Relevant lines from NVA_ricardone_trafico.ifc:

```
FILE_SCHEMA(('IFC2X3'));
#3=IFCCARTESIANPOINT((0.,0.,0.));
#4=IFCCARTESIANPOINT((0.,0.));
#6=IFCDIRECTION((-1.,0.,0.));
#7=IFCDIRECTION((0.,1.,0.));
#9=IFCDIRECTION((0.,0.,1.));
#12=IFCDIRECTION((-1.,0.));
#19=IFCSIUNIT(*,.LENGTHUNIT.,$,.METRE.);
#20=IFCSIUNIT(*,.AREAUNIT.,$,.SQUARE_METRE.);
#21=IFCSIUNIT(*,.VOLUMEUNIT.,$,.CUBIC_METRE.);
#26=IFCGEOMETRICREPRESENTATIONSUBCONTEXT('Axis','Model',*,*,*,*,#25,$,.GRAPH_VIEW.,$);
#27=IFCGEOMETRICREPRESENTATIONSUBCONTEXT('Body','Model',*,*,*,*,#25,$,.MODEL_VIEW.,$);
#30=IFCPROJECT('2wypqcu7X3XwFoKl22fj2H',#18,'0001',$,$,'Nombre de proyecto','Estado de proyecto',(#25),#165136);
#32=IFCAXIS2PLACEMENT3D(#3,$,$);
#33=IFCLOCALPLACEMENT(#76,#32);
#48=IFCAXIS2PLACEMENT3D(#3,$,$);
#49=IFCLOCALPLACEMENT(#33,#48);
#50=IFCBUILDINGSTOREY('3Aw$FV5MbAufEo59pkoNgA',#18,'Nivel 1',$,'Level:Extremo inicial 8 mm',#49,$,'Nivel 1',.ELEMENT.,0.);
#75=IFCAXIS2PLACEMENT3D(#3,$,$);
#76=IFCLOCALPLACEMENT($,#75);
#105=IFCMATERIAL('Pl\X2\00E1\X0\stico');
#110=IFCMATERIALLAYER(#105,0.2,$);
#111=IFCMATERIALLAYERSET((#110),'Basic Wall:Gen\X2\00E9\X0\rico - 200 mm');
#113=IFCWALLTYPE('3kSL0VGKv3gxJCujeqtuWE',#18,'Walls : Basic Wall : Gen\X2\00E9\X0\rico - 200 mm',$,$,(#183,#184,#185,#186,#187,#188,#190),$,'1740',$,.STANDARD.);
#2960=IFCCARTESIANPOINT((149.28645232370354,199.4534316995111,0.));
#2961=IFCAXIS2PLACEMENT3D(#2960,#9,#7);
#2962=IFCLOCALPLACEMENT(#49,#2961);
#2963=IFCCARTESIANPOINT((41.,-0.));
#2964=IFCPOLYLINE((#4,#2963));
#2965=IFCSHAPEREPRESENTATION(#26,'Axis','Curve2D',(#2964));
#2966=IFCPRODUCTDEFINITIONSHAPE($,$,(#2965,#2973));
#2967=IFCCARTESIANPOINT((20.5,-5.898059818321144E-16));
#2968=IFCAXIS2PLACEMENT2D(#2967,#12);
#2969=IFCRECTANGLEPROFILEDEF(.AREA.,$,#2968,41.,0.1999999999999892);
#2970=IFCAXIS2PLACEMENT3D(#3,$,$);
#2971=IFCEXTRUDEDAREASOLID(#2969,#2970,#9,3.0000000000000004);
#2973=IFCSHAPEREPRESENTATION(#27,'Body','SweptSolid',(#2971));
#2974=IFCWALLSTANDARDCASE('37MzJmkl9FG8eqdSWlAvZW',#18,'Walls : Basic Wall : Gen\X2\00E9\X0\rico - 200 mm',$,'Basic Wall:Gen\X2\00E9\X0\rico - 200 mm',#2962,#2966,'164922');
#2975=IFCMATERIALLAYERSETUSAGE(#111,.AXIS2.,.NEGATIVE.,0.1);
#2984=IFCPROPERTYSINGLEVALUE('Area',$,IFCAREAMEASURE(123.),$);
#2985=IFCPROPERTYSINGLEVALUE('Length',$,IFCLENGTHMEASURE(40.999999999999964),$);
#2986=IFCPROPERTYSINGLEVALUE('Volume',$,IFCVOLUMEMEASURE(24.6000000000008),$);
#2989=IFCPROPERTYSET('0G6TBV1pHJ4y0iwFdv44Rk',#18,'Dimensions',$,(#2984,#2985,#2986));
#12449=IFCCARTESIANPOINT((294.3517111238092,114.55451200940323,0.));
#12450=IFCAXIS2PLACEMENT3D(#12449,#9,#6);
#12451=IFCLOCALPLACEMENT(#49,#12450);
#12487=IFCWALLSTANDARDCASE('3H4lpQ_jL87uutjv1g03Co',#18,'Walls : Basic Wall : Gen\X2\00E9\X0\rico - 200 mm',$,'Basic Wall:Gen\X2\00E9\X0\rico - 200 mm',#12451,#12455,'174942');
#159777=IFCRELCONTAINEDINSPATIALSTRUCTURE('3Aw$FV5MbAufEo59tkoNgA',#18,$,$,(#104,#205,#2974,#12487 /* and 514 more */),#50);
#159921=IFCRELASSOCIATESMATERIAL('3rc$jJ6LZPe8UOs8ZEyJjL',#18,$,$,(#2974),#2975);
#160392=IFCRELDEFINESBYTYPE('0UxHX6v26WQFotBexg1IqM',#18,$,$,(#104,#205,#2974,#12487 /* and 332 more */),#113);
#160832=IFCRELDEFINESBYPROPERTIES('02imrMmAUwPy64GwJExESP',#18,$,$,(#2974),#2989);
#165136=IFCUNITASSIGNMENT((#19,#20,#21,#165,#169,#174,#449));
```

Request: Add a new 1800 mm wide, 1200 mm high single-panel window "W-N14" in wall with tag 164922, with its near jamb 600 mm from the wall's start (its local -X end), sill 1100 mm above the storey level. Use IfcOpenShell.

```python
import numpy as np
import ifcopenshell
import ifcopenshell.api.feature
import ifcopenshell.api.geometry
import ifcopenshell.api.pset
import ifcopenshell.api.root
import ifcopenshell.api.spatial
import ifcopenshell.api.type
import ifcopenshell.geom
import ifcopenshell.util.element
import ifcopenshell.util.placement
import ifcopenshell.util.representation
import ifcopenshell.util.shape
import ifcopenshell.util.unit

model = ifcopenshell.open("NVA_ricardone_trafico.ifc")
unit_scale = ifcopenshell.util.unit.calculate_unit_scale(model)
area_scale = ifcopenshell.util.unit.calculate_unit_scale(model, "AREAUNIT")
volume_scale = ifcopenshell.util.unit.calculate_unit_scale(model, "VOLUMEUNIT")
settings = ifcopenshell.geom.settings()


def volume(element):
    """Net volume in cubic metres, openings subtracted."""
    shape = ifcopenshell.geom.create_shape(settings, element)
    return ifcopenshell.util.shape.get_volume(shape.geometry)


wall = model.by_id(2974)
storey = ifcopenshell.util.element.get_container(wall, ifc_class="IfcBuildingStorey")
context = ifcopenshell.util.representation.get_context(model, "Model", "Body", "MODEL_VIEW")
before = volume(wall)

width, height, from_end, sill = 1.8, 1.2, 0.6, 1.1  # metres

# The wall runs along its own X axis, and the end named is its -X end.
wall_shape = ifcopenshell.geom.create_shape(settings, wall)
x, y, z = ifcopenshell.util.shape.get_vertices(wall_shape.geometry).T
start = x.min() + from_end
face, thickness = float(y.min()), float(y.max() - y.min())
wall_matrix = ifcopenshell.util.placement.get_local_placement(wall.ObjectPlacement)
level = ifcopenshell.util.placement.get_local_placement(storey.ObjectPlacement)[2, 3]


def in_wall(x, y):
    """Placement at x, y metres in the wall's axes, at sill height."""
    matrix = wall_matrix.copy()
    matrix[:, 3] = wall_matrix @ np.array([x / unit_scale, y / unit_scale, 0.0, 1.0])
    matrix[2, 3] = level + sill / unit_scale
    return matrix


# Opening: a box that overshoots both wall faces by 50 mm.
opening = ifcopenshell.api.root.create_entity(model, ifc_class="IfcOpeningElement")
box = ifcopenshell.api.geometry.add_wall_representation(
    model, context=context, length=width, height=height, thickness=thickness + 0.1
)
ifcopenshell.api.geometry.assign_representation(model, product=opening, representation=box)
ifcopenshell.api.geometry.edit_object_placement(model, product=opening, matrix=in_wall(start, face - 0.05), is_si=False)
ifcopenshell.api.feature.add_feature(model, feature=opening, element=wall)

window = ifcopenshell.api.root.create_entity(model, ifc_class="IfcWindow", name="W-N14")
window.OverallWidth, window.OverallHeight = width / unit_scale, height / unit_scale
body = ifcopenshell.api.geometry.add_window_representation(
    model,
    context=context,
    overall_width=window.OverallWidth,
    overall_height=window.OverallHeight,
    partition_type="SINGLE_PANEL",
)
ifcopenshell.api.geometry.assign_representation(model, product=window, representation=body)
ifcopenshell.api.spatial.assign_container(model, products=[window], relating_structure=storey)
fills = ifcopenshell.api.feature.add_filling(model, opening=opening, element=window)
fills.OwnerHistory = window.OwnerHistory  # required in IFC2X3

# IFC2X3 keeps the operation on the window style.
style = ifcopenshell.api.root.create_entity(model, ifc_class="IfcWindowStyle", name="W-N14")
style.OperationType, style.ConstructionType = "SINGLE_PANEL", "NOTDEFINED"
style.ParameterTakesPrecedence = style.Sizeable = False
ifcopenshell.api.type.assign_type(model, related_objects=[window], relating_type=style)

# Centre the window in the wall's thickness.
ifcopenshell.api.geometry.edit_object_placement(model, product=window, matrix=in_wall(start, face), is_si=False)
window_shape = ifcopenshell.geom.create_shape(settings, window)
depth = ifcopenshell.util.shape.get_vertices(window_shape.geometry)[:, 1]
offset = face + thickness / 2 - (depth.min() + depth.max()) / 2
ifcopenshell.api.geometry.edit_object_placement(model, product=window, matrix=in_wall(start, offset), is_si=False)

after = volume(wall)

# Update the wall's stored quantities.
pset = model.by_id(ifcopenshell.util.element.get_pset(wall, "Dimensions", should_inherit=False)["id"])
ifcopenshell.api.pset.edit_pset(model, pset=pset, properties={
    "Area": model.create_entity("IfcAreaMeasure", after / thickness / area_scale),
    "Volume": model.create_entity("IfcVolumeMeasure", after / volume_scale),
})

print(f"wall volume {before:.3f} -> {after:.3f} m3")

model.write("NVA_ricardone_trafico_v2.ifc")
```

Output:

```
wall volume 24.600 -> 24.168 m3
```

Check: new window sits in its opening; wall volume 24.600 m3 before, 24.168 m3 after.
